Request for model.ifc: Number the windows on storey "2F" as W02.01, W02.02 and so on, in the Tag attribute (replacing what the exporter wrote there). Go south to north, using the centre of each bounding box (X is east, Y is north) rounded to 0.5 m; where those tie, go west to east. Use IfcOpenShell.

First a look at what the model holds.

```python
import ifcopenshell
import ifcopenshell.util.element
import ifcopenshell.util.placement

model = ifcopenshell.open("model.ifc")
print(model.schema)
storey = next(s for s in model.by_type("IfcBuildingStorey") if s.Name == "2F")
windows = [e for e in ifcopenshell.util.element.get_decomposition(storey) if e.is_a("IfcWindow")]
for e in sorted(windows, key=lambda e: e.id()):
    origin = ifcopenshell.util.placement.get_local_placement(e.ObjectPlacement)[:3, 3]
    print(e.id(), e.Tag, e.Name, origin.round(2) + 0.0, sep=" | ")
```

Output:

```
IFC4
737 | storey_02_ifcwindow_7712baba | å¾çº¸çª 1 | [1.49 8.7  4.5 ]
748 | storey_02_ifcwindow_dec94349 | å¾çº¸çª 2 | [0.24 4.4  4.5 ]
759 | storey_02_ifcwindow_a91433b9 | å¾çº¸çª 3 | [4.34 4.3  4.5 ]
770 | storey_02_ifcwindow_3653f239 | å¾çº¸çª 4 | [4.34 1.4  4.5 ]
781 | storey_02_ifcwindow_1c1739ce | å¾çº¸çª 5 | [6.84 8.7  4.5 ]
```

```python
import ifcopenshell
import ifcopenshell.geom
import ifcopenshell.util.element
import ifcopenshell.util.shape

model = ifcopenshell.open("model.ifc")
settings = ifcopenshell.geom.settings()
settings.set("use-world-coords", True)


def centre(element):
    shape = ifcopenshell.geom.create_shape(settings, element)
    return ifcopenshell.util.shape.get_bbox_centroid(shape.geometry)


storey = next(s for s in model.by_type("IfcBuildingStorey") if s.Name == "2F")
windows = [e for e in ifcopenshell.util.element.get_decomposition(storey) if e.is_a("IfcWindow")]

# Insertion points can sit at a corner or the storey origin, so sort by the geometry (in metres).
centres = {e: centre(e) for e in windows}
windows.sort(key=lambda e: (round(centres[e][1] / 0.5), centres[e][0]))

for i, e in enumerate(windows, start=1):
    number = f"W02.{i:02d}"
    e.Tag = number
    print(e.id(), number)

model.write("model_rev.ifc")
```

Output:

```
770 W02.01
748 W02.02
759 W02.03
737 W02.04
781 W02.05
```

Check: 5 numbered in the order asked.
